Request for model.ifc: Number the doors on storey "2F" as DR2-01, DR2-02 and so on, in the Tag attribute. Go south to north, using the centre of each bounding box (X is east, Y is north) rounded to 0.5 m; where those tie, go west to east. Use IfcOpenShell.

First a look at what the model holds.

```python
import ifcopenshell
import ifcopenshell.util.element
import ifcopenshell.util.placement

model = ifcopenshell.open("model.ifc")
print(model.schema)
storey = next(s for s in model.by_type("IfcBuildingStorey") if s.Name == "2F")
doors = [e for e in ifcopenshell.util.element.get_decomposition(storey) if e.is_a("IfcDoor")]
for e in sorted(doors, key=lambda e: e.id()):
    origin = ifcopenshell.util.placement.get_local_placement(e.ObjectPlacement)[:3, 3]
    print(e.id(), e.Tag, e.Name, origin.round(2) + 0.0, sep=" | ")
```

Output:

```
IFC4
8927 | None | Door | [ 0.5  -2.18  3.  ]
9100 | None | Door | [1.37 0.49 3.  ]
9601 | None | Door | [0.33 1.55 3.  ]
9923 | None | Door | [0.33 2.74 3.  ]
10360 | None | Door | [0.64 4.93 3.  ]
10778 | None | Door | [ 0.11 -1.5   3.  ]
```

```python
import ifcopenshell
import ifcopenshell.geom
import ifcopenshell.util.element
import ifcopenshell.util.shape

model = ifcopenshell.open("model.ifc")
settings = ifcopenshell.geom.settings()
settings.set("use-world-coords", True)


def centre(element):
    shape = ifcopenshell.geom.create_shape(settings, element)
    return ifcopenshell.util.shape.get_bbox_centroid(shape.geometry)


storey = next(s for s in model.by_type("IfcBuildingStorey") if s.Name == "2F")
doors = [e for e in ifcopenshell.util.element.get_decomposition(storey) if e.is_a("IfcDoor")]

# Insertion points can sit at a corner or the storey origin, so sort by the geometry (in metres).
centres = {e: centre(e) for e in doors}
doors.sort(key=lambda e: (round(centres[e][1] / 0.5), centres[e][0]))

for i, e in enumerate(doors, start=1):
    number = f"DR2-{i:02d}"
    e.Tag = number
    print(e.id(), number)

model.write("model_v2.ifc")
```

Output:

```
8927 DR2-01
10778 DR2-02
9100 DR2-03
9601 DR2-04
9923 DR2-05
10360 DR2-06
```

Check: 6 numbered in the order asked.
